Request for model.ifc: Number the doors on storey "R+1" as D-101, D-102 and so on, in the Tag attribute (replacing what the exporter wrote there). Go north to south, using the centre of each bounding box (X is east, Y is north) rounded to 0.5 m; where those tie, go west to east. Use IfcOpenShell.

First a look at what the model holds.

```python
import ifcopenshell
import ifcopenshell.util.element
import ifcopenshell.util.placement

model = ifcopenshell.open("model.ifc")
print(model.schema)
storey = next(s for s in model.by_type("IfcBuildingStorey") if s.Name == "R+1")
doors = [e for e in ifcopenshell.util.element.get_decomposition(storey) if e.is_a("IfcDoor")]
for e in sorted(doors, key=lambda e: e.id()):
    origin = ifcopenshell.util.placement.get_local_placement(e.ObjectPlacement)[:3, 3]
    print(e.id(), e.Tag, e.Name, origin.round(2) + 0.0, sep=" | ")
```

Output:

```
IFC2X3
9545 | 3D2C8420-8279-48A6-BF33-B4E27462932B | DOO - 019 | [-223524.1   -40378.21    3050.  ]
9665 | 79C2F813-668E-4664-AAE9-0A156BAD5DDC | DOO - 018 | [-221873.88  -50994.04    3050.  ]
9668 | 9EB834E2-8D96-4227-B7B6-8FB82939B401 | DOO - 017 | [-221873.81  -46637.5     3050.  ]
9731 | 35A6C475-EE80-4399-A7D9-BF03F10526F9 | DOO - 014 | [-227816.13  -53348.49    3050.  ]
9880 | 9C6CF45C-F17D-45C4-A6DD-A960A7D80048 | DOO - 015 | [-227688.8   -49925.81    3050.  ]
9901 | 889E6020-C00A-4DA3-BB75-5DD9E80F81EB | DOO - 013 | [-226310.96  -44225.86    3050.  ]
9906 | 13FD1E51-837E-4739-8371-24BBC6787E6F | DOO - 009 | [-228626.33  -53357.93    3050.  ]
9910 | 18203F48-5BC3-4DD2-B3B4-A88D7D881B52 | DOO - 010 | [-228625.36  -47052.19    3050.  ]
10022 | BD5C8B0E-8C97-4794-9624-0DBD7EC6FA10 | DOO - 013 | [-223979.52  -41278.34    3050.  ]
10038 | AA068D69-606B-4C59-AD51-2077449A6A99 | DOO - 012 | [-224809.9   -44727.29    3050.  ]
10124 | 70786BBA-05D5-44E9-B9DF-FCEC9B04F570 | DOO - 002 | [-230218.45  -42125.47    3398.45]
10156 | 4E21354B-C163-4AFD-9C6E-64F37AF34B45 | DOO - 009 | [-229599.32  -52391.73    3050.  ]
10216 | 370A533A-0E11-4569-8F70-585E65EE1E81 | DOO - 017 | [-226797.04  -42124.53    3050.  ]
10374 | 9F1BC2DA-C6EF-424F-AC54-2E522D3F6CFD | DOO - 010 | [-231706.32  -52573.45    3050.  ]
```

```python
import ifcopenshell
import ifcopenshell.geom
import ifcopenshell.util.element
import ifcopenshell.util.shape

model = ifcopenshell.open("model.ifc")
settings = ifcopenshell.geom.settings()
settings.set("use-world-coords", True)


def centre(element):
    shape = ifcopenshell.geom.create_shape(settings, element)
    return ifcopenshell.util.shape.get_bbox_centroid(shape.geometry)


storey = next(s for s in model.by_type("IfcBuildingStorey") if s.Name == "R+1")
doors = [e for e in ifcopenshell.util.element.get_decomposition(storey) if e.is_a("IfcDoor")]

# Insertion points can sit at a corner or the storey origin, so sort by the geometry (in metres).
centres = {e: centre(e) for e in doors}
doors.sort(key=lambda e: (-round(centres[e][1] / 0.5), centres[e][0]))

for i, e in enumerate(doors, start=1):
    number = f"D-1{i:02d}"
    e.Tag = number
    print(e.id(), number)

model.write("model_v2.ifc")
```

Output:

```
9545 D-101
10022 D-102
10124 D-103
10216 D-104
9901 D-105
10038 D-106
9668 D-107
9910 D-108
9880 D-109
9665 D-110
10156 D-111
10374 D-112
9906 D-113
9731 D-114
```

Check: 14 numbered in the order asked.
